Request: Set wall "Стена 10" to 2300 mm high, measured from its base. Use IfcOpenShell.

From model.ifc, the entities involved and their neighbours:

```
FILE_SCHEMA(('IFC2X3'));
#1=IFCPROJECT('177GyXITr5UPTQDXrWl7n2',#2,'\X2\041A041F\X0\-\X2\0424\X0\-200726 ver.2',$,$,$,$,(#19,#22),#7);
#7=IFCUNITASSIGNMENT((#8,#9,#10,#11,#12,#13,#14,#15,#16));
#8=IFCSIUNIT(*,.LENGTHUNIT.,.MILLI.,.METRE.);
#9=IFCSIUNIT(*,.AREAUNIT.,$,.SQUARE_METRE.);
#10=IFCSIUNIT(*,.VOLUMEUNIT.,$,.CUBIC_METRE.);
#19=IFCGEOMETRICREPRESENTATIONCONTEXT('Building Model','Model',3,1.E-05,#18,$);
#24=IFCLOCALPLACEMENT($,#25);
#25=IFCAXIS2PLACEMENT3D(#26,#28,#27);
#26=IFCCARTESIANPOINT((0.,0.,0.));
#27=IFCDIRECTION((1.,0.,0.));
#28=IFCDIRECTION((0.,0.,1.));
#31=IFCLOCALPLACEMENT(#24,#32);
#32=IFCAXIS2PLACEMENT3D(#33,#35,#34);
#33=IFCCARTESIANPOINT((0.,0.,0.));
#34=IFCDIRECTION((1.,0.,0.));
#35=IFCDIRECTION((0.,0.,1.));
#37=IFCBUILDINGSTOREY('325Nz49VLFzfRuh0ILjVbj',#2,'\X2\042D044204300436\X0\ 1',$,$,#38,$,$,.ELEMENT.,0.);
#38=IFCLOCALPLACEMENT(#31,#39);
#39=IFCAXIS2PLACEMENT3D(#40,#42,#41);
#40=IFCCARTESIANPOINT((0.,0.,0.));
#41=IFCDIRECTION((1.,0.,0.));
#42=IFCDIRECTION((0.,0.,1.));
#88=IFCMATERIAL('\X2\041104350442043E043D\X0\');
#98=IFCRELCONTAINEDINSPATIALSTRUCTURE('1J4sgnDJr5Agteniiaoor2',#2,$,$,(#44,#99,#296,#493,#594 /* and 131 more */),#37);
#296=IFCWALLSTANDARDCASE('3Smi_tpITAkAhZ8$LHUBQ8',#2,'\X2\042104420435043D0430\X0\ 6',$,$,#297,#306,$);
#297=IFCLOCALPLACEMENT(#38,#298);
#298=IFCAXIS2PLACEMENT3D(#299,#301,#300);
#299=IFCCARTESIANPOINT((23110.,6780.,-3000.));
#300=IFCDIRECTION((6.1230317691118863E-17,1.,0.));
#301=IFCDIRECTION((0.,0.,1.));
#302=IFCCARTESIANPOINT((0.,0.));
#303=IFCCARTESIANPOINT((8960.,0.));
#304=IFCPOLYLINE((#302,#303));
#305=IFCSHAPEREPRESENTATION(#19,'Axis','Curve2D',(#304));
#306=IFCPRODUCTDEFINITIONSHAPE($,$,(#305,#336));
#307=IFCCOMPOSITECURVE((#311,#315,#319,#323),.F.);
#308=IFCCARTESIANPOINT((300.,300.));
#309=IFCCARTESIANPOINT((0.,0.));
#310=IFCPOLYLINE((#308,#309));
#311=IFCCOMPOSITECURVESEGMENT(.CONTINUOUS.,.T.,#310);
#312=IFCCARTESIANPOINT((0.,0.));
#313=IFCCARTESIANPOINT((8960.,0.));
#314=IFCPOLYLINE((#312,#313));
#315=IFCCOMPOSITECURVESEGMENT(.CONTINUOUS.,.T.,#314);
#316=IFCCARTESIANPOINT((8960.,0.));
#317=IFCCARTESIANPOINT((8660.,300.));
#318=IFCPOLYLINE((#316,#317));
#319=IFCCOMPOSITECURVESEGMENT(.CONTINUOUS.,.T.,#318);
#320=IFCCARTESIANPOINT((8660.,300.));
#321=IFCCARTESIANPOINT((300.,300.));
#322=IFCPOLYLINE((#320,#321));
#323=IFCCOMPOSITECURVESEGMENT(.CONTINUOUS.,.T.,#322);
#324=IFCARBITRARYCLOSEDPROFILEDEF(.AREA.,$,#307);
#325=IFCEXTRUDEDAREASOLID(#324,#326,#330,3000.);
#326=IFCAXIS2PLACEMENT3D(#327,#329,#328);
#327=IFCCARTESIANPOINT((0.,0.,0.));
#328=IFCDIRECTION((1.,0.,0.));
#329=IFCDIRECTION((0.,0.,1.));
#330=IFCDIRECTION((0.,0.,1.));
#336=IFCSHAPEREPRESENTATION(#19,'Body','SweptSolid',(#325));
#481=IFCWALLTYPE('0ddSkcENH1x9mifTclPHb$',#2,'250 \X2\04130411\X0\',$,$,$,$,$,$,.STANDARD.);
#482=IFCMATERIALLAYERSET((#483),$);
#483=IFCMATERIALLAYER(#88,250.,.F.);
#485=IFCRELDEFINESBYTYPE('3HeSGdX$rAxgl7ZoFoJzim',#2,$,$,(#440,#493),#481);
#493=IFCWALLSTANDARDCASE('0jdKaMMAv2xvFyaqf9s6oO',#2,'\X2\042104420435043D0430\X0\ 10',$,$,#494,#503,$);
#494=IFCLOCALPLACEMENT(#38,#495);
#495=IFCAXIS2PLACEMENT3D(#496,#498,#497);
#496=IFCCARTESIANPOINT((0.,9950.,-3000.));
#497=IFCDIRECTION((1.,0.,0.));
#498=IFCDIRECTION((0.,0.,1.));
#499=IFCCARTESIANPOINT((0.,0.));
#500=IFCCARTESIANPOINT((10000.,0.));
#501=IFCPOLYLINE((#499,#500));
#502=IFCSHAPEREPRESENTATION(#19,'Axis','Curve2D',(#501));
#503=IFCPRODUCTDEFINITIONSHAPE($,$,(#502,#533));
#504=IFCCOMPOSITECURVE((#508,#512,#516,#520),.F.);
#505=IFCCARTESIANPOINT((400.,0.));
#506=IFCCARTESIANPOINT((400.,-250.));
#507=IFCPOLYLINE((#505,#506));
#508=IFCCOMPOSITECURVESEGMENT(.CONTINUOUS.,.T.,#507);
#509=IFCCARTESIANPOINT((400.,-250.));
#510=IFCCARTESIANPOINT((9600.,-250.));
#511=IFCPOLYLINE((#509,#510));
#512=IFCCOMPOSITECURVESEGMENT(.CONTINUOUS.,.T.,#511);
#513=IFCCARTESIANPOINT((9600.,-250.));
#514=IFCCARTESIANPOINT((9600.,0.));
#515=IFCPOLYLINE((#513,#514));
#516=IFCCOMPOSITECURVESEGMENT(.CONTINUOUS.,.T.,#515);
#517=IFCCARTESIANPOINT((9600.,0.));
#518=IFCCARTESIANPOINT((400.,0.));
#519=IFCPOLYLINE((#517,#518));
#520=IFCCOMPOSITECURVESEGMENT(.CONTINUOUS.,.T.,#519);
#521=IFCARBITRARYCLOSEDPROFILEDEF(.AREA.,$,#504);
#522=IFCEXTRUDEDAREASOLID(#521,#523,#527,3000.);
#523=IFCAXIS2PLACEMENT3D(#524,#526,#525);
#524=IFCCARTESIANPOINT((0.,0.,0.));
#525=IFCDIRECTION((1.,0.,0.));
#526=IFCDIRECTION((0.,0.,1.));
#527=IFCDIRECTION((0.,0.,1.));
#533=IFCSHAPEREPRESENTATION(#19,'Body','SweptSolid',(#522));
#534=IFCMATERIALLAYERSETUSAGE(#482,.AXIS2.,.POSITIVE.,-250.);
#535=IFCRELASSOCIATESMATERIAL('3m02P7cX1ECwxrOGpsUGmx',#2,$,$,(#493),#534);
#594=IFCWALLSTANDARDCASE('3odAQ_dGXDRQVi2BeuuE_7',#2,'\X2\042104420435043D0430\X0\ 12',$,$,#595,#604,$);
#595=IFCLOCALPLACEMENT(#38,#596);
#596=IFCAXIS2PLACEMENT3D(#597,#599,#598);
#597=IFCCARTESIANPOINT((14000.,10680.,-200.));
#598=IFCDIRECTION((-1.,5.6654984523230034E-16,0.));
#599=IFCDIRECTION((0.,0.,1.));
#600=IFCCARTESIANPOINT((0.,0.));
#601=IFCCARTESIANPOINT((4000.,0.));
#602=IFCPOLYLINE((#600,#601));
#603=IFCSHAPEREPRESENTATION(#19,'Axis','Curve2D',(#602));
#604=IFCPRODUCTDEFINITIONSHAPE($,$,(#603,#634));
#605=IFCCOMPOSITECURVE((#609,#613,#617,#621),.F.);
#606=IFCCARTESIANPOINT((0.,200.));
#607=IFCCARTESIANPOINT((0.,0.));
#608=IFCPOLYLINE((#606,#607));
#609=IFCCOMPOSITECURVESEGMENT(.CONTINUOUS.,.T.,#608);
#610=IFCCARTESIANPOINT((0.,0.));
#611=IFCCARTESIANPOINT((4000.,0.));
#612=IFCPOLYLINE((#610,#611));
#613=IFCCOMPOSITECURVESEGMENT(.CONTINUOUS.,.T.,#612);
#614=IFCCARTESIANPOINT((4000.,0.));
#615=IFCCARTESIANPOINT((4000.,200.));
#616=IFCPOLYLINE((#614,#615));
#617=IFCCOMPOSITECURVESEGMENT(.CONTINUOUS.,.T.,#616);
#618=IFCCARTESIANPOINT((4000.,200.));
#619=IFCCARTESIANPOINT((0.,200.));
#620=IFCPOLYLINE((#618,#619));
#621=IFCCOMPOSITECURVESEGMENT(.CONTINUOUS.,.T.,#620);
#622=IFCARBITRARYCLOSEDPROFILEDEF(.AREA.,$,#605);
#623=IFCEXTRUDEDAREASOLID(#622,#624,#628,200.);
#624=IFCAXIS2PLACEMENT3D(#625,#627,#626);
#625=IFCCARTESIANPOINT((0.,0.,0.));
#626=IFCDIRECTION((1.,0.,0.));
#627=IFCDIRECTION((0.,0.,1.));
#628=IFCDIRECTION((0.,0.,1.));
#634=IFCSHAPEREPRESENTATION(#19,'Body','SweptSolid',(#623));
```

```python
import ifcopenshell
import ifcopenshell.geom
import ifcopenshell.util.shape
import ifcopenshell.util.unit

model = ifcopenshell.open("model.ifc")
unit_scale = ifcopenshell.util.unit.calculate_unit_scale(model)
settings = ifcopenshell.geom.settings()


def volume(element):
    """Net volume in cubic metres, openings subtracted."""
    shape = ifcopenshell.geom.create_shape(settings, element)
    return ifcopenshell.util.shape.get_volume(shape.geometry)


wall = model.by_guid("0jdKaMMAv2xvFyaqf9s6oO")
before = volume(wall)

body = next(r for r in wall.Representation.Representations if r.RepresentationIdentifier == "Body")
solid = body.Items[0]
old_height = solid.Depth
solid.Depth = 2.3 / unit_scale
after = volume(wall)

print(f"height {old_height:g} -> {solid.Depth:g}, volume {before:.3f} -> {after:.3f} m3")

model.write("model_v2.ifc")
```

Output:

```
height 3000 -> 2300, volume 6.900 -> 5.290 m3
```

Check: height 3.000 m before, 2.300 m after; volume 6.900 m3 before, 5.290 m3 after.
